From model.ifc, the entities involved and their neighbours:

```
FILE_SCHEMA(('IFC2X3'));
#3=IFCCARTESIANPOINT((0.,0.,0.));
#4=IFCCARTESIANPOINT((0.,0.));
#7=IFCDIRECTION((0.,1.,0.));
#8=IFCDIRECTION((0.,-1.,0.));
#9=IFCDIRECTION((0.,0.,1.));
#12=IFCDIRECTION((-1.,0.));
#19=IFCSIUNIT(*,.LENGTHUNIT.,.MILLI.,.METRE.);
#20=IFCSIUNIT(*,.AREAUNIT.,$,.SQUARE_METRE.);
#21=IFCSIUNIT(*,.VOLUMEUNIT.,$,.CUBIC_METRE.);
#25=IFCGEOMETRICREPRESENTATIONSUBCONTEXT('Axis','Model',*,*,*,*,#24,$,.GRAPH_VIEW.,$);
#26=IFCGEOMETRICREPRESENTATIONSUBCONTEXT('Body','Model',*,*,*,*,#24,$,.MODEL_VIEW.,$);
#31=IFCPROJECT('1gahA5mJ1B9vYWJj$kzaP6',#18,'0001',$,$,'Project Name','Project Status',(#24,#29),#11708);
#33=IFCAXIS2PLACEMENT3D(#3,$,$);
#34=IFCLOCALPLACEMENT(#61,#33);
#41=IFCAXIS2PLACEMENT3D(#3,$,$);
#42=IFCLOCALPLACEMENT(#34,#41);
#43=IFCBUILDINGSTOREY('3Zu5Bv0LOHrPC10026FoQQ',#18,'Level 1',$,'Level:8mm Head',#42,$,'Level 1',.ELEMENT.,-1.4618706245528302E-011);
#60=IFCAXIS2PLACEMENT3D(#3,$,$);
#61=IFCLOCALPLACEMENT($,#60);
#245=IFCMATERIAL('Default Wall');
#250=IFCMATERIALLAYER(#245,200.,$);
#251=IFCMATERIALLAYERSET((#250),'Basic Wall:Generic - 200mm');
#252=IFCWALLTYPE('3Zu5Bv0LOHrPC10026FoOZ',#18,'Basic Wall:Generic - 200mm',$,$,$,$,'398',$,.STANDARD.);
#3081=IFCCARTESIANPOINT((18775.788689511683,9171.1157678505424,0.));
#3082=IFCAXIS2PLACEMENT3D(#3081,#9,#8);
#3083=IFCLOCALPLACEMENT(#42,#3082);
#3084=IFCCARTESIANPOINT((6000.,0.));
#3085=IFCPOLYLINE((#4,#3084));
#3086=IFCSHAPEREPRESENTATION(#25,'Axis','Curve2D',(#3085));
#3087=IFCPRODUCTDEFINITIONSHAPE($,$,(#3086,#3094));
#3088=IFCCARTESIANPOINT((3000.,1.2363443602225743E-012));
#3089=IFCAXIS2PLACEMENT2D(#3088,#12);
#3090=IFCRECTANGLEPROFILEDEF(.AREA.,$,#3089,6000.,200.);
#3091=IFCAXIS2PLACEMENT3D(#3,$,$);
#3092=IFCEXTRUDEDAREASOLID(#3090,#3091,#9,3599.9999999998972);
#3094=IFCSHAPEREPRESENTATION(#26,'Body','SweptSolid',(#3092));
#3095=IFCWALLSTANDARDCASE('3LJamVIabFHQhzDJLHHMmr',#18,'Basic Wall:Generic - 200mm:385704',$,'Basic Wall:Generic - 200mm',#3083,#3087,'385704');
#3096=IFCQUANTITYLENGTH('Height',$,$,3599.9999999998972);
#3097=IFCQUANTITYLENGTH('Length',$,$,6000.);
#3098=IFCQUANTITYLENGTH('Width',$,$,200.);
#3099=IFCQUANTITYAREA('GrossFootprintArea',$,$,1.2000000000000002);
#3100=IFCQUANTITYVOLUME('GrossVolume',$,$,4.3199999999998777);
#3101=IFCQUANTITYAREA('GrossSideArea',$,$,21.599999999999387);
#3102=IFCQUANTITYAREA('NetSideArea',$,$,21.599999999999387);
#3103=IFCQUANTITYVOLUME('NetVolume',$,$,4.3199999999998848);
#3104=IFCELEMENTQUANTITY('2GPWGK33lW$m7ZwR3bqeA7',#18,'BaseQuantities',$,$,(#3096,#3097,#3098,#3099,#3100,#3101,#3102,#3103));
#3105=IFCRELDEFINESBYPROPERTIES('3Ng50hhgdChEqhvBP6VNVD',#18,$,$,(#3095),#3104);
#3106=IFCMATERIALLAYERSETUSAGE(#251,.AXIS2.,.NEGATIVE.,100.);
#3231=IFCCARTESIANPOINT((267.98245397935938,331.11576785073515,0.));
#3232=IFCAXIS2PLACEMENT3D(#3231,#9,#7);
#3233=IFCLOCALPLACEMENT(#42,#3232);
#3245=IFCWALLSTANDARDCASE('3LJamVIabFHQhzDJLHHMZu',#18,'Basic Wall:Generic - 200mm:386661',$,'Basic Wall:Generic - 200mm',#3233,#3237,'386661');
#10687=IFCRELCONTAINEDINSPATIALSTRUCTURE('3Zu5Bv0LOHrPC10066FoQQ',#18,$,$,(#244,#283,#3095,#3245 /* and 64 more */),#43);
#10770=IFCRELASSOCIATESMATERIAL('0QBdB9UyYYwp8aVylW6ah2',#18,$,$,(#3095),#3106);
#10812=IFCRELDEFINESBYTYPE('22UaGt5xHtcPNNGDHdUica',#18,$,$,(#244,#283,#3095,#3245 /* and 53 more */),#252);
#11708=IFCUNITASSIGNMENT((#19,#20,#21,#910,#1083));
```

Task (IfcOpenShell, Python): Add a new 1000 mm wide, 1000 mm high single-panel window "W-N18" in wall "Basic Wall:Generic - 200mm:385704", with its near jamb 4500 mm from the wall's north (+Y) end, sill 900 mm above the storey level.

```python
import numpy as np
import ifcopenshell
import ifcopenshell.api.feature
import ifcopenshell.api.geometry
import ifcopenshell.api.pset
import ifcopenshell.api.root
import ifcopenshell.api.spatial
import ifcopenshell.api.type
import ifcopenshell.geom
import ifcopenshell.util.element
import ifcopenshell.util.placement
import ifcopenshell.util.representation
import ifcopenshell.util.shape
import ifcopenshell.util.unit

model = ifcopenshell.open("model.ifc")
unit_scale = ifcopenshell.util.unit.calculate_unit_scale(model)
area_scale = ifcopenshell.util.unit.calculate_unit_scale(model, "AREAUNIT")
volume_scale = ifcopenshell.util.unit.calculate_unit_scale(model, "VOLUMEUNIT")
settings = ifcopenshell.geom.settings()


def volume(element):
    """Net volume in cubic metres, openings subtracted."""
    shape = ifcopenshell.geom.create_shape(settings, element)
    return ifcopenshell.util.shape.get_volume(shape.geometry)


wall = model.by_guid("3LJamVIabFHQhzDJLHHMmr")
storey = ifcopenshell.util.element.get_container(wall, ifc_class="IfcBuildingStorey")
context = ifcopenshell.util.representation.get_context(model, "Model", "Body", "MODEL_VIEW")
before = volume(wall)

width, height, from_end, sill = 1, 1, 4.5, 0.9  # metres

# The wall runs along its own X axis, and the end named is its -X end.
wall_shape = ifcopenshell.geom.create_shape(settings, wall)
x, y, z = ifcopenshell.util.shape.get_vertices(wall_shape.geometry).T
start = x.min() + from_end
face, thickness = float(y.min()), float(y.max() - y.min())
wall_matrix = ifcopenshell.util.placement.get_local_placement(wall.ObjectPlacement)
level = ifcopenshell.util.placement.get_local_placement(storey.ObjectPlacement)[2, 3]


def in_wall(x, y):
    """Placement at x, y metres in the wall's axes, at sill height."""
    matrix = wall_matrix.copy()
    matrix[:, 3] = wall_matrix @ np.array([x / unit_scale, y / unit_scale, 0.0, 1.0])
    matrix[2, 3] = level + sill / unit_scale
    return matrix


# Opening: a box that overshoots both wall faces by 50 mm.
opening = ifcopenshell.api.root.create_entity(model, ifc_class="IfcOpeningElement")
box = ifcopenshell.api.geometry.add_wall_representation(
    model, context=context, length=width, height=height, thickness=thickness + 0.1
)
ifcopenshell.api.geometry.assign_representation(model, product=opening, representation=box)
ifcopenshell.api.geometry.edit_object_placement(model, product=opening, matrix=in_wall(start, face - 0.05), is_si=False)
ifcopenshell.api.feature.add_feature(model, feature=opening, element=wall)

window = ifcopenshell.api.root.create_entity(model, ifc_class="IfcWindow", name="W-N18")
window.OverallWidth, window.OverallHeight = width / unit_scale, height / unit_scale
body = ifcopenshell.api.geometry.add_window_representation(
    model,
    context=context,
    overall_width=window.OverallWidth,
    overall_height=window.OverallHeight,
    partition_type="SINGLE_PANEL",
)
ifcopenshell.api.geometry.assign_representation(model, product=window, representation=body)
ifcopenshell.api.spatial.assign_container(model, products=[window], relating_structure=storey)
fills = ifcopenshell.api.feature.add_filling(model, opening=opening, element=window)
fills.OwnerHistory = window.OwnerHistory  # required in IFC2X3

# IFC2X3 keeps the operation on the window style.
style = ifcopenshell.api.root.create_entity(model, ifc_class="IfcWindowStyle", name="W-N18")
style.OperationType, style.ConstructionType = "SINGLE_PANEL", "NOTDEFINED"
style.ParameterTakesPrecedence = style.Sizeable = False
ifcopenshell.api.type.assign_type(model, related_objects=[window], relating_type=style)

# Centre the window in the wall's thickness.
ifcopenshell.api.geometry.edit_object_placement(model, product=window, matrix=in_wall(start, face), is_si=False)
window_shape = ifcopenshell.geom.create_shape(settings, window)
depth = ifcopenshell.util.shape.get_vertices(window_shape.geometry)[:, 1]
offset = face + thickness / 2 - (depth.min() + depth.max()) / 2
ifcopenshell.api.geometry.edit_object_placement(model, product=window, matrix=in_wall(start, offset), is_si=False)

after = volume(wall)

# Update the wall's stored quantities.
qto = model.by_id(ifcopenshell.util.element.get_pset(wall, "BaseQuantities", should_inherit=False)["id"])
ifcopenshell.api.pset.edit_qto(model, qto=qto, properties={
    "NetSideArea": after / thickness / area_scale,
    "NetVolume": after / volume_scale,
})

print(f"wall volume {before:.3f} -> {after:.3f} m3")

model.write("model_edited.ifc")
```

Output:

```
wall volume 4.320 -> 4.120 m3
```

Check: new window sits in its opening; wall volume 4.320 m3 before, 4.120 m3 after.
